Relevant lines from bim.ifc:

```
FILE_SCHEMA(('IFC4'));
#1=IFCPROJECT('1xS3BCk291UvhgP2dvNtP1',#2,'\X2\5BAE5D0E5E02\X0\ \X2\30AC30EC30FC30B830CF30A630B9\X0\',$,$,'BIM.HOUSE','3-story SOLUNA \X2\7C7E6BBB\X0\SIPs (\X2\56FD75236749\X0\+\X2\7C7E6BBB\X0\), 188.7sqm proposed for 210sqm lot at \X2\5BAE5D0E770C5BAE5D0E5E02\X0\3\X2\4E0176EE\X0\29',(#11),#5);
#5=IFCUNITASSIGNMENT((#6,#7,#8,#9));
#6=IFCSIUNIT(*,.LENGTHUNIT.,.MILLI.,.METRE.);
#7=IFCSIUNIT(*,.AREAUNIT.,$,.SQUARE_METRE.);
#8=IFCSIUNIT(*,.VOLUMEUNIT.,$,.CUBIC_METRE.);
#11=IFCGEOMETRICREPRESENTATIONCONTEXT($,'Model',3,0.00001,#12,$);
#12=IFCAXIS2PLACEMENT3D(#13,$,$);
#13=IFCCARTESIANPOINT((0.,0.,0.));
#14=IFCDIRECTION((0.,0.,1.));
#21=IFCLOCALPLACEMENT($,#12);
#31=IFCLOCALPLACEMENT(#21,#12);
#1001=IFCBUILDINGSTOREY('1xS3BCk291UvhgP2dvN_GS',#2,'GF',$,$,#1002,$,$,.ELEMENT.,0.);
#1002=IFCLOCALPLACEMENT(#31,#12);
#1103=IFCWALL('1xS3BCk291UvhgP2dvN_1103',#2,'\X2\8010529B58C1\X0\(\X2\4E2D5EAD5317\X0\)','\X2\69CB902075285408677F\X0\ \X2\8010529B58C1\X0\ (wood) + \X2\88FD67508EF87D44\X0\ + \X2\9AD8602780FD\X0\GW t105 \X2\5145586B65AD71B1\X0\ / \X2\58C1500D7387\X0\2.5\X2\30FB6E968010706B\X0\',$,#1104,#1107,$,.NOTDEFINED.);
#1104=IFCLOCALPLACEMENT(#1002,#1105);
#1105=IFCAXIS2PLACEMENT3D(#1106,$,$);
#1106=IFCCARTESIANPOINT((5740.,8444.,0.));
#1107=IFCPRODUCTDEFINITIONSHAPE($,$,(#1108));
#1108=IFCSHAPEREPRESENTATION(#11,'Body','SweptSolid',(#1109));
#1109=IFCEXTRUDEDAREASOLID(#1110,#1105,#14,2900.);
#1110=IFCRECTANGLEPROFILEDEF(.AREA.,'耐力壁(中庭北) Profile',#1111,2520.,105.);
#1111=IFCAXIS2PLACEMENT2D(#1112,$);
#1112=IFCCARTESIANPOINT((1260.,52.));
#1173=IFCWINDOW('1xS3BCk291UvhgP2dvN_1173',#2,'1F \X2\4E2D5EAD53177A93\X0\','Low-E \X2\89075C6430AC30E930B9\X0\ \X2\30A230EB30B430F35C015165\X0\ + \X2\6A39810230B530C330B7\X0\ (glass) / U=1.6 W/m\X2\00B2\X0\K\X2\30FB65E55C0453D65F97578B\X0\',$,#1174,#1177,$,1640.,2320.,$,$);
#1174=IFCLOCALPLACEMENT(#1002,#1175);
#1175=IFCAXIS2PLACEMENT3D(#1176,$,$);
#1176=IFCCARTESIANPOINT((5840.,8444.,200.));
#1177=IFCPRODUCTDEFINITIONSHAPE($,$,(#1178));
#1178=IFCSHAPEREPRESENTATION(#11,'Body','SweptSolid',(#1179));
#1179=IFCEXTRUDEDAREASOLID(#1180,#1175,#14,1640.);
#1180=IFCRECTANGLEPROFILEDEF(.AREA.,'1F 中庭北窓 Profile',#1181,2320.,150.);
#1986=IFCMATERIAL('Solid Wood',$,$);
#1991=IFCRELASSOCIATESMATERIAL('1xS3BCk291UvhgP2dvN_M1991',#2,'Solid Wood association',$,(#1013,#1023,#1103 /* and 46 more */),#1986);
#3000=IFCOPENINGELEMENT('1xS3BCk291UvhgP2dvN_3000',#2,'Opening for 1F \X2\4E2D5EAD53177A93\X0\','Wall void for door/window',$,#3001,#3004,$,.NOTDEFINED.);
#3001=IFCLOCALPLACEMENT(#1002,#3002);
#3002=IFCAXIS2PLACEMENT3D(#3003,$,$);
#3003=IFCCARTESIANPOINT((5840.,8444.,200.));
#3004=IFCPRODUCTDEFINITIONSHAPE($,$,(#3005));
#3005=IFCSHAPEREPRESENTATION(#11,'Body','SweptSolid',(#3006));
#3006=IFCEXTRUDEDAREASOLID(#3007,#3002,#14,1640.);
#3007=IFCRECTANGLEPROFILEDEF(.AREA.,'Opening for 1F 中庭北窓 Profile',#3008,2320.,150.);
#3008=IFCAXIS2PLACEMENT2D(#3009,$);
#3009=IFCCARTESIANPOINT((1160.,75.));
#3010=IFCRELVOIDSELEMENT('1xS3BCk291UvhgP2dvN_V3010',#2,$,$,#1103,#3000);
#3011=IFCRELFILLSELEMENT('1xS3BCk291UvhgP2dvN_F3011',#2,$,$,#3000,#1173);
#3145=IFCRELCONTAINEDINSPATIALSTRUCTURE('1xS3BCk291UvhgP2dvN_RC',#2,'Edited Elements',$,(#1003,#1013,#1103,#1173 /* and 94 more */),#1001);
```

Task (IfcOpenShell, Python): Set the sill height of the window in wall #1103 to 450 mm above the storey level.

```python
import numpy as np
import ifcopenshell
import ifcopenshell.api.geometry
import ifcopenshell.geom
import ifcopenshell.util.element
import ifcopenshell.util.placement
import ifcopenshell.util.shape
import ifcopenshell.util.unit

model = ifcopenshell.open("bim.ifc")
unit_scale = ifcopenshell.util.unit.calculate_unit_scale(model)

window = model.by_guid("1xS3BCk291UvhgP2dvN_1173")
opening = window.FillsVoids[0].RelatingOpeningElement
storey = ifcopenshell.util.element.get_container(window, ifc_class="IfcBuildingStorey")
level = ifcopenshell.util.placement.get_local_placement(storey.ObjectPlacement)[2, 3]

# The opening's origin need not be at the sill, so measure its lowest point.
shape = ifcopenshell.geom.create_shape(ifcopenshell.geom.settings(), opening)
bottom = ifcopenshell.util.shape.get_shape_bottom_elevation(shape, shape.geometry) / unit_scale
dz = level + 0.45 / unit_scale - bottom

shift = np.array([0.0, 0.0, dz])
# The window is not placed relative to its opening, so move both.
for product in (opening, window):
    matrix = ifcopenshell.util.placement.get_local_placement(product.ObjectPlacement)
    matrix[:3, 3] += shift
    ifcopenshell.api.geometry.edit_object_placement(model, product=product, matrix=matrix, is_si=False)

print(f"moved by {dz * unit_scale:+.3f} m")

model.write("bim-out.ifc")
```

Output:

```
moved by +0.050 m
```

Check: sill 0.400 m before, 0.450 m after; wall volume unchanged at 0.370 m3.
